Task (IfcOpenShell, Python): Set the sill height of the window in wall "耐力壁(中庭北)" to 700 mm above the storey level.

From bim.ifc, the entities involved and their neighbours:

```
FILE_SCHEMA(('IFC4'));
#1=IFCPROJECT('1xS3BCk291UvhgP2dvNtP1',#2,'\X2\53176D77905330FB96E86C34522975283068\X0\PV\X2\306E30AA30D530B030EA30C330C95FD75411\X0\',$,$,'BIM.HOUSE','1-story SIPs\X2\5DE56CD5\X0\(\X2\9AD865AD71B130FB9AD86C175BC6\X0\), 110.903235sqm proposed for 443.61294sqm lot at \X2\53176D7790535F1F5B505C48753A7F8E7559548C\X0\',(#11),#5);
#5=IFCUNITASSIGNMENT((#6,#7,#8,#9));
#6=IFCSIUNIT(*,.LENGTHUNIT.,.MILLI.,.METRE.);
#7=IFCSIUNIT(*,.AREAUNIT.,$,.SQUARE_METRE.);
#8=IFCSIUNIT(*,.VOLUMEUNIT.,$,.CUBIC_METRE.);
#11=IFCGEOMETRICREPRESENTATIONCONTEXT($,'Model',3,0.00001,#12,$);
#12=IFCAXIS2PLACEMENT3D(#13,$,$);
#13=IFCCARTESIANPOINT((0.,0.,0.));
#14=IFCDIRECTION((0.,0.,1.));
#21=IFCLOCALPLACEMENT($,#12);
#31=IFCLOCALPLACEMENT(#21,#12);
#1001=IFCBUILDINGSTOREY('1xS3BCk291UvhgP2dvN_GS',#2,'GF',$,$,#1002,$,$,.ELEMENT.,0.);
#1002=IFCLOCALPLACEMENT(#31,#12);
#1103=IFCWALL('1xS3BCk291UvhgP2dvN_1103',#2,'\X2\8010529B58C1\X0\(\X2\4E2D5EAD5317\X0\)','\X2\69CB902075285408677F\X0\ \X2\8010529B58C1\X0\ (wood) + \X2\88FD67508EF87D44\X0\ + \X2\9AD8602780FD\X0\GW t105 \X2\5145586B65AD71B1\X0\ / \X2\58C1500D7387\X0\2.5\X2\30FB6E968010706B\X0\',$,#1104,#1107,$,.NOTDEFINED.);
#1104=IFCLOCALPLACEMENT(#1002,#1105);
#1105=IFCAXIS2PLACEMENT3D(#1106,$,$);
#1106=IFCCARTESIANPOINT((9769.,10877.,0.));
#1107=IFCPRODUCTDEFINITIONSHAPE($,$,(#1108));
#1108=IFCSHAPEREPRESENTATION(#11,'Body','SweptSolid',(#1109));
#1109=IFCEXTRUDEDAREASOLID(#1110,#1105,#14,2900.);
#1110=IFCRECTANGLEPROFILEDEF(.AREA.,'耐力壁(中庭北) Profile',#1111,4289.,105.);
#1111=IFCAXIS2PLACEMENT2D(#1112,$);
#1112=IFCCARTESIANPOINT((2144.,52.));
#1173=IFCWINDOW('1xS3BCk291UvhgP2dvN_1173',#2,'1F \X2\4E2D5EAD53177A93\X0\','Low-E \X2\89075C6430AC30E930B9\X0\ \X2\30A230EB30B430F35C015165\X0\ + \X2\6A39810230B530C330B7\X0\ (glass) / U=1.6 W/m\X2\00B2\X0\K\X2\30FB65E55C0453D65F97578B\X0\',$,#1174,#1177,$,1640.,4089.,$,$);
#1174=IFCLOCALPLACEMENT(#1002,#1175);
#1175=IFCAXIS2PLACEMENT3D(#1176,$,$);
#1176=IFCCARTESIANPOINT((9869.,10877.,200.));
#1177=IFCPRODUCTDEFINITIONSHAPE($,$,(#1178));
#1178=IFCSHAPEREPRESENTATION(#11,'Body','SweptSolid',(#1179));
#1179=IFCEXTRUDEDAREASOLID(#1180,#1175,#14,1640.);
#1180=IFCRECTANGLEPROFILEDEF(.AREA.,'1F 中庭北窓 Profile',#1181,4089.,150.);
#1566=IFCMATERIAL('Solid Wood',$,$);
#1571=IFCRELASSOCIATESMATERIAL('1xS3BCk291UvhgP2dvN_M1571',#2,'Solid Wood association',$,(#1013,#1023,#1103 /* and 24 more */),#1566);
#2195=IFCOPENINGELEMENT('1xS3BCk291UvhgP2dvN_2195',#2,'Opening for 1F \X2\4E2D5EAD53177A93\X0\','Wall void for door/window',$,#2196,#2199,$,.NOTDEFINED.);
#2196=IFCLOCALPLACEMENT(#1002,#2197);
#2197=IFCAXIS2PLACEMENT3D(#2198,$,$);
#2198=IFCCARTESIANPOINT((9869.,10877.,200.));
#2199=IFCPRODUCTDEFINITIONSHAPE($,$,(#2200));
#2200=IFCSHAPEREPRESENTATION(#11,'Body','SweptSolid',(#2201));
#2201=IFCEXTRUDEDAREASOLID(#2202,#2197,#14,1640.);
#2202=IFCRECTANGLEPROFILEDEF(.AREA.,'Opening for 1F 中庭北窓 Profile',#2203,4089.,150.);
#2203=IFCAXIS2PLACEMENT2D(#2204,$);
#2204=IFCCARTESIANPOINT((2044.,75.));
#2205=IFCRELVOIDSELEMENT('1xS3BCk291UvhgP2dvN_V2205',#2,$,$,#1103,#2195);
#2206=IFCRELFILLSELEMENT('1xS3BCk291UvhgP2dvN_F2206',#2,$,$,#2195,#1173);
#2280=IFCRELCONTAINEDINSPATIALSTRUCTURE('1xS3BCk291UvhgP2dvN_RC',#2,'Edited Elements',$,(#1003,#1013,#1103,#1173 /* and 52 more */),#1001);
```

```python
import numpy as np
import ifcopenshell
import ifcopenshell.api.geometry
import ifcopenshell.geom
import ifcopenshell.util.element
import ifcopenshell.util.placement
import ifcopenshell.util.shape
import ifcopenshell.util.unit

model = ifcopenshell.open("bim.ifc")
unit_scale = ifcopenshell.util.unit.calculate_unit_scale(model)

window = model.by_guid("1xS3BCk291UvhgP2dvN_1173")
opening = window.FillsVoids[0].RelatingOpeningElement
storey = ifcopenshell.util.element.get_container(window, ifc_class="IfcBuildingStorey")
level = ifcopenshell.util.placement.get_local_placement(storey.ObjectPlacement)[2, 3]

# The opening's origin need not be at the sill, so measure its lowest point.
shape = ifcopenshell.geom.create_shape(ifcopenshell.geom.settings(), opening)
bottom = ifcopenshell.util.shape.get_shape_bottom_elevation(shape, shape.geometry) / unit_scale
dz = level + 0.7 / unit_scale - bottom

shift = np.array([0.0, 0.0, dz])
# The window is not placed relative to its opening, so move both.
for product in (opening, window):
    matrix = ifcopenshell.util.placement.get_local_placement(product.ObjectPlacement)
    matrix[:3, 3] += shift
    ifcopenshell.api.geometry.edit_object_placement(model, product=product, matrix=matrix, is_si=False)

print(f"moved by {dz * unit_scale:+.3f} m")

model.write("bim_v2.ifc")
```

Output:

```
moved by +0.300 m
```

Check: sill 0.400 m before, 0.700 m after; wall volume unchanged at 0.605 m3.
